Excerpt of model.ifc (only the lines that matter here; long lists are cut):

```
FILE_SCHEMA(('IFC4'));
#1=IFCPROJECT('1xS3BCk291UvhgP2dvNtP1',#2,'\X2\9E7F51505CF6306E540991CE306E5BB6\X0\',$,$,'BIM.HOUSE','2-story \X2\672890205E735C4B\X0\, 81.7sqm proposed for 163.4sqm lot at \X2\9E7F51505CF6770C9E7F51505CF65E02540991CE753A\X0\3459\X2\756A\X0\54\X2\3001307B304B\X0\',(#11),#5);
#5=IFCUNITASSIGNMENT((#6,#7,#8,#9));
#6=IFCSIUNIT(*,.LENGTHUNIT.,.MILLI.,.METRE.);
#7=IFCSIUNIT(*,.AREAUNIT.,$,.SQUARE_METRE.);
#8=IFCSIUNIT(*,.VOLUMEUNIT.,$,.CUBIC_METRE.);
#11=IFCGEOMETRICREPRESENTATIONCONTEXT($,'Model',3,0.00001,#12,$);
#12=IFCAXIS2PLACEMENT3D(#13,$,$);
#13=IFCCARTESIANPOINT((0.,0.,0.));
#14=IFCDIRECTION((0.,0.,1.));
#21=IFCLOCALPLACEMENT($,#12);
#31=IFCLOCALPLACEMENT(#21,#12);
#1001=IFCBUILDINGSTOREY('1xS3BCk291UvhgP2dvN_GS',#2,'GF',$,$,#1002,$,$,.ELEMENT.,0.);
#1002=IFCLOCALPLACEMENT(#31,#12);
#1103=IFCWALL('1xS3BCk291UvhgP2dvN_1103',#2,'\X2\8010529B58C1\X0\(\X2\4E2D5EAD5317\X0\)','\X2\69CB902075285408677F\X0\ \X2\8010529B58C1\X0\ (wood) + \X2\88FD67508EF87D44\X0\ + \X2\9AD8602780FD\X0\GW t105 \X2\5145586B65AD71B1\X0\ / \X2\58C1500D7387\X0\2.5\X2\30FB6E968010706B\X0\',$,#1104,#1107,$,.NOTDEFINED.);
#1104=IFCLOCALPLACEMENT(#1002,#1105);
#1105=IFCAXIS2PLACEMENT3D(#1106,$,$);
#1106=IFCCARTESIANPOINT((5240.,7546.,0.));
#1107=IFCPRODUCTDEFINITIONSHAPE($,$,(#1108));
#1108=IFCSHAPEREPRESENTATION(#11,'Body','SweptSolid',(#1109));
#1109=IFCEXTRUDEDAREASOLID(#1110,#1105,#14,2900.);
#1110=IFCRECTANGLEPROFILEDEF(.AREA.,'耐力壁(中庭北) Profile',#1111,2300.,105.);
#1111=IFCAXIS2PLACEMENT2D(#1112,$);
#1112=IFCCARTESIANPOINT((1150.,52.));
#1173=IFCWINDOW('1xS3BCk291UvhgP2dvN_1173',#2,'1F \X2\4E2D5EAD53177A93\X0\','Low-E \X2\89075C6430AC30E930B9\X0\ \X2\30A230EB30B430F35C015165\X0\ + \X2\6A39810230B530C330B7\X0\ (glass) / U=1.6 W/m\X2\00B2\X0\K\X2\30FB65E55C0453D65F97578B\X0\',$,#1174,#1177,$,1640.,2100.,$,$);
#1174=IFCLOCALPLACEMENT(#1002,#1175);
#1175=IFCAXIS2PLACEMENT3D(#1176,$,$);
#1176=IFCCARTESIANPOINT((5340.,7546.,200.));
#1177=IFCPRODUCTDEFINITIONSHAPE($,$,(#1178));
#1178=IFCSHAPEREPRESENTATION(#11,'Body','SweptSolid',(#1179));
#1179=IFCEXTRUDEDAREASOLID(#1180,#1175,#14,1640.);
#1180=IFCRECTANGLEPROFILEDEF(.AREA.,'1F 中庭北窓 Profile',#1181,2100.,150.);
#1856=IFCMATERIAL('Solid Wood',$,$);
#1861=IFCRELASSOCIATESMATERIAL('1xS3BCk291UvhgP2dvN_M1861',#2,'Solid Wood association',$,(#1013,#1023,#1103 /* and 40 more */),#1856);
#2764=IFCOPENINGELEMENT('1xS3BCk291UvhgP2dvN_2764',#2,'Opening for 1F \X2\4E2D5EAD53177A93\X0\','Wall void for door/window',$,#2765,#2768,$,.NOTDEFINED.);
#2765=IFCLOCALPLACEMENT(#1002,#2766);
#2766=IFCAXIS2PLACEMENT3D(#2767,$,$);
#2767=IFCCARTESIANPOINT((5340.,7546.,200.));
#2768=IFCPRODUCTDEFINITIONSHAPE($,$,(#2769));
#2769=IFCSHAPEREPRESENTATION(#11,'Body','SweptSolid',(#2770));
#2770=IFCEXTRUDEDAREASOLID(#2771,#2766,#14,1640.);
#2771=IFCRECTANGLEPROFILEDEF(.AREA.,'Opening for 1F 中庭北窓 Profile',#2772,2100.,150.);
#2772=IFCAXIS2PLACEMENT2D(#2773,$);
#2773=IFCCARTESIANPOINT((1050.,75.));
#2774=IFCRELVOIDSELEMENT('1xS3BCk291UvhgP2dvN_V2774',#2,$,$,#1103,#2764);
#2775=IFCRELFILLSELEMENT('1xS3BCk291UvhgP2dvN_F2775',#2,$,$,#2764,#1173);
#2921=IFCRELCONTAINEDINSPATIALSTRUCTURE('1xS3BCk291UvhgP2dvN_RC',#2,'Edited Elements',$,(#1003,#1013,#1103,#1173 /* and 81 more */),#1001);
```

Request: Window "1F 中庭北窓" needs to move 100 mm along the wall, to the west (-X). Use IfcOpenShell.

```python
import ifcopenshell
import ifcopenshell.api.geometry
import ifcopenshell.util.placement
import ifcopenshell.util.unit

model = ifcopenshell.open("model.ifc")
unit_scale = ifcopenshell.util.unit.calculate_unit_scale(model)

window = model.by_guid("1xS3BCk291UvhgP2dvN_1173")
opening = window.FillsVoids[0].RelatingOpeningElement
wall = opening.VoidsElements[0].RelatingBuildingElement

wall_matrix = ifcopenshell.util.placement.get_local_placement(wall.ObjectPlacement)
shift = wall_matrix[:3, 0] * -0.1 / unit_scale
before = ifcopenshell.util.placement.get_local_placement(window.ObjectPlacement)[:3, 3].copy()

# The window is not placed relative to its opening, so move both.
for product in (opening, window):
    matrix = ifcopenshell.util.placement.get_local_placement(product.ObjectPlacement)
    matrix[:3, 3] += shift
    ifcopenshell.api.geometry.edit_object_placement(model, product=product, matrix=matrix, is_si=False)

after = ifcopenshell.util.placement.get_local_placement(window.ObjectPlacement)[:3, 3]
print("window moved by", (after - before).round(3) + 0.0)

model.write("model_edited.ifc")
```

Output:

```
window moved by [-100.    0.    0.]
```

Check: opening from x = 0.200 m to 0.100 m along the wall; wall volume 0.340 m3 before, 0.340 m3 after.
